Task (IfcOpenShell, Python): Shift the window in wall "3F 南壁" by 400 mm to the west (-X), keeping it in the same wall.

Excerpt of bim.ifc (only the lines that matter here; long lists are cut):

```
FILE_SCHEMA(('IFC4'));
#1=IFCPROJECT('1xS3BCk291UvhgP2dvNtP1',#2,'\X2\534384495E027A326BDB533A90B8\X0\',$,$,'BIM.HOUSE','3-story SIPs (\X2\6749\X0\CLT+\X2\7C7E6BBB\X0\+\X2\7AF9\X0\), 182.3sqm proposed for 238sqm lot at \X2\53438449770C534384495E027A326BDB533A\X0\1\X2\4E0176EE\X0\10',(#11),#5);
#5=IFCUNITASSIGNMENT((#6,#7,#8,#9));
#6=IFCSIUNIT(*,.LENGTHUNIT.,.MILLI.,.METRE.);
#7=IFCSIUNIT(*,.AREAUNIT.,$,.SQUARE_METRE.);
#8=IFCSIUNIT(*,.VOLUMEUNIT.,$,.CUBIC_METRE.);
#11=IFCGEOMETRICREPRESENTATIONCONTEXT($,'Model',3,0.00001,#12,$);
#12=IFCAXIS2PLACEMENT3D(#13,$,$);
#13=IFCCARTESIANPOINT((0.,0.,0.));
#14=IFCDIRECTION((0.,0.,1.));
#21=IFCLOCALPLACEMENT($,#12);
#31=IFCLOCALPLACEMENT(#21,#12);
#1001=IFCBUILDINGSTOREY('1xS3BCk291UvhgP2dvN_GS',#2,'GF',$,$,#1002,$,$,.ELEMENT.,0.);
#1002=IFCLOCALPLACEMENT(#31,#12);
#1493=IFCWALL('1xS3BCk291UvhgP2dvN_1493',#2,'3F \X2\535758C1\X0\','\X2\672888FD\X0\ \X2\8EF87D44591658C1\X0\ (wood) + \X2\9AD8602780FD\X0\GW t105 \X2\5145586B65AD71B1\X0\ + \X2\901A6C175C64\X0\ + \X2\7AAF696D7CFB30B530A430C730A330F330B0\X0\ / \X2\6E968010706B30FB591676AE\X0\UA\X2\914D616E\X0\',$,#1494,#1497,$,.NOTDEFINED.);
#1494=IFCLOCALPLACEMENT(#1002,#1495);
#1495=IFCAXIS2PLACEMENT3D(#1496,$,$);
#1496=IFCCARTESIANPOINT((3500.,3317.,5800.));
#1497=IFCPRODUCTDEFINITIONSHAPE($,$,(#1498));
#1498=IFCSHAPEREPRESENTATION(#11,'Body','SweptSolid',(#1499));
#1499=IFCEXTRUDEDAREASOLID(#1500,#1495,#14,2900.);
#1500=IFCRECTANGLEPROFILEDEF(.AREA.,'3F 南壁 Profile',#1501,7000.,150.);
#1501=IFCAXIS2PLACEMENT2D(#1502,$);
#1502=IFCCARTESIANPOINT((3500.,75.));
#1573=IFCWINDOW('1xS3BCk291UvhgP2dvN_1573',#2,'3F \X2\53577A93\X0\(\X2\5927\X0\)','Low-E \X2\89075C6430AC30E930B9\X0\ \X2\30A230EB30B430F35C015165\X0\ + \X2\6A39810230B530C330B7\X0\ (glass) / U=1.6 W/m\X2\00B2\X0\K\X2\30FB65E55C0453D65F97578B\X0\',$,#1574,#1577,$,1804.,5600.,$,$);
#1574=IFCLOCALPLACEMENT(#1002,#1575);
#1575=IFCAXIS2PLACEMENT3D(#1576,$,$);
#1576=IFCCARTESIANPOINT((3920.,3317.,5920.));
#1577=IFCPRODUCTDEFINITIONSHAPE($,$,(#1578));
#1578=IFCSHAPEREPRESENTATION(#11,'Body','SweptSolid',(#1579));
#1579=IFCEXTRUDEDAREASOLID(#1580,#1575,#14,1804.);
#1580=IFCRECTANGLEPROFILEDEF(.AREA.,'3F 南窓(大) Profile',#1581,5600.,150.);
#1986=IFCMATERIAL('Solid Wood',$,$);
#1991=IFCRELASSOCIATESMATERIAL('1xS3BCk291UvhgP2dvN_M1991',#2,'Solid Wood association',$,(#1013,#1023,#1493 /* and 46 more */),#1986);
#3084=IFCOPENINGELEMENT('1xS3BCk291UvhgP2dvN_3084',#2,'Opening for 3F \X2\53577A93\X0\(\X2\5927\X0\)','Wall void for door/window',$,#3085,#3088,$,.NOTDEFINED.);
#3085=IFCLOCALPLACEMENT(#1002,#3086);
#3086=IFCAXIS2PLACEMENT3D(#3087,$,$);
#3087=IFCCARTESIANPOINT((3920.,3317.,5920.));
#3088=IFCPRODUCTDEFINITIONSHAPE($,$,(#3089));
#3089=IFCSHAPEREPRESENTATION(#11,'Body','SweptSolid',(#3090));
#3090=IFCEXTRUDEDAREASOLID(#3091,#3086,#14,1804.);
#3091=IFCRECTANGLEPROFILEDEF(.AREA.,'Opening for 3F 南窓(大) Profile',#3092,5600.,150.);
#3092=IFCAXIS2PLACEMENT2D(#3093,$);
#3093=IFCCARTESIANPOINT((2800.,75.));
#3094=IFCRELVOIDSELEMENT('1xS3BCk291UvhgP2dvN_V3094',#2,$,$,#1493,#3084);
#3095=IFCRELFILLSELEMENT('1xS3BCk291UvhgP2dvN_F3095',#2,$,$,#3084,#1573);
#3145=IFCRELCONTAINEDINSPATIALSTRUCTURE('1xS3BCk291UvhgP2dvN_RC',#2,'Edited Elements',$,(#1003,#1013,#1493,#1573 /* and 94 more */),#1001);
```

```python
import ifcopenshell
import ifcopenshell.api.geometry
import ifcopenshell.util.placement

model = ifcopenshell.open("bim.ifc")

window = model.by_guid("1xS3BCk291UvhgP2dvN_1573")
opening = window.FillsVoids[0].RelatingOpeningElement
wall = opening.VoidsElements[0].RelatingBuildingElement

wall_matrix = ifcopenshell.util.placement.get_local_placement(wall.ObjectPlacement)
shift = wall_matrix[:3, 0] * -400.0
before = ifcopenshell.util.placement.get_local_placement(window.ObjectPlacement)[:3, 3].copy()

# The window is not placed relative to its opening, so move both.
for product in (opening, window):
    matrix = ifcopenshell.util.placement.get_local_placement(product.ObjectPlacement)
    matrix[:3, 3] += shift
    ifcopenshell.api.geometry.edit_object_placement(model, product=product, matrix=matrix, is_si=False)

after = ifcopenshell.util.placement.get_local_placement(window.ObjectPlacement)[:3, 3]
print("window moved by", (after - before).round(3) + 0.0)

model.write("bim_rev.ifc")
```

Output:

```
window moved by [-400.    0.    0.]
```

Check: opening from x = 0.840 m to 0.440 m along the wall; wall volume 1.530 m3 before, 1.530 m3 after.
